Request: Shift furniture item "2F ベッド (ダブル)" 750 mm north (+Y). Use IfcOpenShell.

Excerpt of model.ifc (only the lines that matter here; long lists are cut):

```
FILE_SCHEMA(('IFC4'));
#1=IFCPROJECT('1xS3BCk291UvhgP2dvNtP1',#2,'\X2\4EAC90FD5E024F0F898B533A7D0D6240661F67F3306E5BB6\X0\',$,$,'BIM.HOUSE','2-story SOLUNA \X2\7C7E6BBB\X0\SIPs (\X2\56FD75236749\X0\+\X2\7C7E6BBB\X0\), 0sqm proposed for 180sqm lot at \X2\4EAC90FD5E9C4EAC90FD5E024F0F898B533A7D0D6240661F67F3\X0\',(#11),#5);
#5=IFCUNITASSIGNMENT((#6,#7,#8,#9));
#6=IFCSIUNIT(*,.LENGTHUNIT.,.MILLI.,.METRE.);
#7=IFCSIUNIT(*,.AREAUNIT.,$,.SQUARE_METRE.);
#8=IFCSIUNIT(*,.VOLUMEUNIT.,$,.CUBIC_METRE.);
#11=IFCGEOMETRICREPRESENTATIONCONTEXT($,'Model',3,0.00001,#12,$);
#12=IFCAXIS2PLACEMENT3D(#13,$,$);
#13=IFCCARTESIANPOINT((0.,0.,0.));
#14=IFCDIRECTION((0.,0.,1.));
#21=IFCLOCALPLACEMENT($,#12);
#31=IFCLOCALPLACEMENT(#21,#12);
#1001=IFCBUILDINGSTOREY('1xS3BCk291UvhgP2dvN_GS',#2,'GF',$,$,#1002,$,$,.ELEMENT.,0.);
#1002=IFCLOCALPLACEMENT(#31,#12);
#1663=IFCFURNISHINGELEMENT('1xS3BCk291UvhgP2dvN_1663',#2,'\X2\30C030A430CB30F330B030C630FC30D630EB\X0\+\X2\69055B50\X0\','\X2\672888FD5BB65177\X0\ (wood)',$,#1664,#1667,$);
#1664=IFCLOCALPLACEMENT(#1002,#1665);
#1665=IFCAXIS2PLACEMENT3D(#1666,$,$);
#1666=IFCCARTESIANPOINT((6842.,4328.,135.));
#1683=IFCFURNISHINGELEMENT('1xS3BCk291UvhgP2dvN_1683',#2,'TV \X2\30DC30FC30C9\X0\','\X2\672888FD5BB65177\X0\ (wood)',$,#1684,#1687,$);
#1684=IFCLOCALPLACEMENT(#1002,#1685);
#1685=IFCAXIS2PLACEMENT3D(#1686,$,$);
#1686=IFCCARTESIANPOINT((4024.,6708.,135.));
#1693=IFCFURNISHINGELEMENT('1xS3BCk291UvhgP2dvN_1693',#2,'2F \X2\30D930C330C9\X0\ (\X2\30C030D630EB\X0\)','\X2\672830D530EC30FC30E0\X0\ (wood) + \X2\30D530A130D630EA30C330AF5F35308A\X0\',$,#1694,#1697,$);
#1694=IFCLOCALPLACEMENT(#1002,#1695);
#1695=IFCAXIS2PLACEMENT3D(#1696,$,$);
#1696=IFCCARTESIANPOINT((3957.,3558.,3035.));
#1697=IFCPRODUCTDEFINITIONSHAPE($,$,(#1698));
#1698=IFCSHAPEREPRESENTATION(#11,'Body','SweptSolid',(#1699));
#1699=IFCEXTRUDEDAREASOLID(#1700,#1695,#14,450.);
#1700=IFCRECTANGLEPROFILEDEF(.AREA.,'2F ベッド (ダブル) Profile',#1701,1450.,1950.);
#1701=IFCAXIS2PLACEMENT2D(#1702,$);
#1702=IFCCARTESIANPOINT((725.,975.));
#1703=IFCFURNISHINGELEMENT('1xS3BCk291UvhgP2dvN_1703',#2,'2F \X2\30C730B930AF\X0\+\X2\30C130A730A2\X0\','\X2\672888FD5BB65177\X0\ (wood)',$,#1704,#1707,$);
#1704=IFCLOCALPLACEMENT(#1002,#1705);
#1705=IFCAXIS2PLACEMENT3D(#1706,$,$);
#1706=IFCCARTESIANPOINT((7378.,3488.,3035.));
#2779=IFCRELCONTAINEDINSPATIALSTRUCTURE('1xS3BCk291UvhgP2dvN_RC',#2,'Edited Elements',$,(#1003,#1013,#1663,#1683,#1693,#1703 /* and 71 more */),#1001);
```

```python
import ifcopenshell
import ifcopenshell.api.geometry
import ifcopenshell.util.placement
import ifcopenshell.util.unit

model = ifcopenshell.open("model.ifc")
unit_scale = ifcopenshell.util.unit.calculate_unit_scale(model)

item = model.by_guid("1xS3BCk291UvhgP2dvN_1693")
matrix = ifcopenshell.util.placement.get_local_placement(item.ObjectPlacement)
matrix[1, 3] += 0.75 / unit_scale
ifcopenshell.api.geometry.edit_object_placement(model, product=item, matrix=matrix, is_si=False)

print(ifcopenshell.util.placement.get_local_placement(item.ObjectPlacement).round(3) + 0.0)

model.write("model-out.ifc")
```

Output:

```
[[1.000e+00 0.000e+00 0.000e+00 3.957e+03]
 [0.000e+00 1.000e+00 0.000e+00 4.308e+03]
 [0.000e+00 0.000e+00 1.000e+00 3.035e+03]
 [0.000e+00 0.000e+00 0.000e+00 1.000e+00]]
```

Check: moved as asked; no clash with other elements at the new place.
